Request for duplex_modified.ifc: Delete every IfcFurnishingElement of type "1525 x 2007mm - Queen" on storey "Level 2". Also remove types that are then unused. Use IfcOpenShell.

First a look at what the model holds.

```python
import ifcopenshell
import ifcopenshell.util.element

model = ifcopenshell.open("duplex_modified.ifc")
print(model.schema)
storey = next(s for s in model.by_type("IfcBuildingStorey") if s.Name == "Level 2")
furniture = [e for e in ifcopenshell.util.element.get_decomposition(storey) if e.is_a("IfcFurnishingElement")]
seen = {}
for e in furniture:
    element_type = ifcopenshell.util.element.get_type(e)
    name = element_type.Name if element_type not in (None, e) else None
    seen[name] = seen.get(name, 0) + 1
for name, count in sorted(seen.items(), key=str):
    print(count, "x", name)
```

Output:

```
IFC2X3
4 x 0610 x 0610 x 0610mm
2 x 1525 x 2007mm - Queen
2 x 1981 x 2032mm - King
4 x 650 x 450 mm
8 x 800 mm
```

```python
import ifcopenshell
import ifcopenshell.api.root
import ifcopenshell.util.element

model = ifcopenshell.open("duplex_modified.ifc")

storey = next(s for s in model.by_type("IfcBuildingStorey") if s.Name == "Level 2")
furniture = [e for e in ifcopenshell.util.element.get_decomposition(storey) if e.is_a("IfcFurnishingElement")]
targets = [e for e in furniture if (t := ifcopenshell.util.element.get_type(e)) not in (None, e) and t.Name == "1525 x 2007mm - Queen"]
types = {ifcopenshell.util.element.get_type(e) for e in targets} - {None, *targets}

for e in targets:
    ifcopenshell.api.root.remove_product(model, product=e)
print(len(targets), "removed")

unused = [t for t in types if not ifcopenshell.util.element.get_types(t)]
for t in unused:
    ifcopenshell.api.root.remove_product(model, product=t)
print(len(unused), "unused types removed")

model.write("duplex_modified_updated.ifc")
```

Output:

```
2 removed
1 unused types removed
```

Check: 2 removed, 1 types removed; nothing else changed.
